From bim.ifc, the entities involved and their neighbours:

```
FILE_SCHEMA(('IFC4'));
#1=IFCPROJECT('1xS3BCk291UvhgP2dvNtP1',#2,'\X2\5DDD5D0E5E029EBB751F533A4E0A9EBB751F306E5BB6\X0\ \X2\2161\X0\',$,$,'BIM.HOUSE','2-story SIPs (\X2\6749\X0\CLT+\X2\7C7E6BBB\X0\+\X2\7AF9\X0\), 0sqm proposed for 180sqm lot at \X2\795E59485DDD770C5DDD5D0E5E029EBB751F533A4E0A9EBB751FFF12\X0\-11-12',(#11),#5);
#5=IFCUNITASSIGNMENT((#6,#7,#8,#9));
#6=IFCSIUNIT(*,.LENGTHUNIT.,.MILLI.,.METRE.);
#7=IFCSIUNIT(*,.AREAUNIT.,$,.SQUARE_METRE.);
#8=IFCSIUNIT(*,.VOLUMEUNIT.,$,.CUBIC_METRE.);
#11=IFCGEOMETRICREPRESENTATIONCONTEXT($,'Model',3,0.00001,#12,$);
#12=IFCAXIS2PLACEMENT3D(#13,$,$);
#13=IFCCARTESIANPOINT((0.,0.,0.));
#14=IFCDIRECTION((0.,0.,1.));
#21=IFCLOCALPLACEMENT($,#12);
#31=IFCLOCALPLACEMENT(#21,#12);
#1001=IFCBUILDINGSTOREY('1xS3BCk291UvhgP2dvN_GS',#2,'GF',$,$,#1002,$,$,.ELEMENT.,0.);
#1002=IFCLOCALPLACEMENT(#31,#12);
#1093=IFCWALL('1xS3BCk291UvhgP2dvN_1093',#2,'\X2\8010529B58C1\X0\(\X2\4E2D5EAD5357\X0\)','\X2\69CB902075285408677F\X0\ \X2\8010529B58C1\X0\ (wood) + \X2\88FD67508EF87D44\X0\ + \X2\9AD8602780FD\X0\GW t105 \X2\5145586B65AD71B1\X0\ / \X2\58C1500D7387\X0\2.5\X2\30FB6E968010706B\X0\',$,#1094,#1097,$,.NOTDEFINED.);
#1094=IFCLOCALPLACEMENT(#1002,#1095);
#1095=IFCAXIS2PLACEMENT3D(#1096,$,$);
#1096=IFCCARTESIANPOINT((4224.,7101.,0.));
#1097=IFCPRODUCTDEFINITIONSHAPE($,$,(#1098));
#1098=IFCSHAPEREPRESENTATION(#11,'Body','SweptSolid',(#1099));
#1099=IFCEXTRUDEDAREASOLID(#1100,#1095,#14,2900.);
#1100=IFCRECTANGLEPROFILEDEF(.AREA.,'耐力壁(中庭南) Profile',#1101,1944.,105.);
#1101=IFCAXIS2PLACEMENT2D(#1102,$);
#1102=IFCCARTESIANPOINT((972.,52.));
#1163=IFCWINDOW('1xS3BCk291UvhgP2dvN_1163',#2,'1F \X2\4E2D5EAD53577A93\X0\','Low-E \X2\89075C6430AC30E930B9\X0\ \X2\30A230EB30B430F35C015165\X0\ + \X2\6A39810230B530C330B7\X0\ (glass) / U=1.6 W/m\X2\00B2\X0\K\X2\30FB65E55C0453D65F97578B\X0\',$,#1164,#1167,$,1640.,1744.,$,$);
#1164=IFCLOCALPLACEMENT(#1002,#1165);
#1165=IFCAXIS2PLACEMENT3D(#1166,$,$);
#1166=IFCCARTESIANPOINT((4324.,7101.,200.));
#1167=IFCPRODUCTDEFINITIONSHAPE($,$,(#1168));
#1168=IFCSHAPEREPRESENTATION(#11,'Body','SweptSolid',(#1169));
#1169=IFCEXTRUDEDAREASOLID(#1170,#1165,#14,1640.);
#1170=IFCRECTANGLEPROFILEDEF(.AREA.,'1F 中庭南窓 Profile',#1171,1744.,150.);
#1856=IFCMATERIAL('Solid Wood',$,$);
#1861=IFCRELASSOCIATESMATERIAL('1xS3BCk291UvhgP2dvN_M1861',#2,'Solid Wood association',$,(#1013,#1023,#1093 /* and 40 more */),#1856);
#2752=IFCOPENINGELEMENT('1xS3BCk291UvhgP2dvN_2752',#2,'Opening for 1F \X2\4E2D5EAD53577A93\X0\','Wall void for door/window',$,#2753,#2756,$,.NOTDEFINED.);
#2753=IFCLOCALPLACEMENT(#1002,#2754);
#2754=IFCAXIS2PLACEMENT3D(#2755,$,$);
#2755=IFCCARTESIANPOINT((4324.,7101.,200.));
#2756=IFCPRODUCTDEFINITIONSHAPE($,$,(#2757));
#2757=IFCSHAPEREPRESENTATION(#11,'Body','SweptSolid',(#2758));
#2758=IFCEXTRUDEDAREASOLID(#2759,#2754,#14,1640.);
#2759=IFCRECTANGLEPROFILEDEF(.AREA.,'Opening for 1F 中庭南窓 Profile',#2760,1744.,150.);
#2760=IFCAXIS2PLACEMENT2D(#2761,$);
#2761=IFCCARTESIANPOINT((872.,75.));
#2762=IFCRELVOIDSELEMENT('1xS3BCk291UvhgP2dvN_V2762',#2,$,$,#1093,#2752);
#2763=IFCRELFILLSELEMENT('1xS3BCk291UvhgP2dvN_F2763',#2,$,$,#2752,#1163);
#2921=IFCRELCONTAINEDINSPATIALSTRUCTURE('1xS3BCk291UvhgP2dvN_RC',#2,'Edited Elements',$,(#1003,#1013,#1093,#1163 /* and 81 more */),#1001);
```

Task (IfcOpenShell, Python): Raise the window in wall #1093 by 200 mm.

```python
import numpy as np
import ifcopenshell
import ifcopenshell.api.geometry
import ifcopenshell.util.placement
import ifcopenshell.util.unit

model = ifcopenshell.open("bim.ifc")
unit_scale = ifcopenshell.util.unit.calculate_unit_scale(model)

window = model.by_id(1163)
opening = window.FillsVoids[0].RelatingOpeningElement
dz = 200.0

shift = np.array([0.0, 0.0, dz])
# The window is not placed relative to its opening, so move both.
for product in (opening, window):
    matrix = ifcopenshell.util.placement.get_local_placement(product.ObjectPlacement)
    matrix[:3, 3] += shift
    ifcopenshell.api.geometry.edit_object_placement(model, product=product, matrix=matrix, is_si=False)

print(f"moved by {dz * unit_scale:+.3f} m")

model.write("bim_updated.ifc")
```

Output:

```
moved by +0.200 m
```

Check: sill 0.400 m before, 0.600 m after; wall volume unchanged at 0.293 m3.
